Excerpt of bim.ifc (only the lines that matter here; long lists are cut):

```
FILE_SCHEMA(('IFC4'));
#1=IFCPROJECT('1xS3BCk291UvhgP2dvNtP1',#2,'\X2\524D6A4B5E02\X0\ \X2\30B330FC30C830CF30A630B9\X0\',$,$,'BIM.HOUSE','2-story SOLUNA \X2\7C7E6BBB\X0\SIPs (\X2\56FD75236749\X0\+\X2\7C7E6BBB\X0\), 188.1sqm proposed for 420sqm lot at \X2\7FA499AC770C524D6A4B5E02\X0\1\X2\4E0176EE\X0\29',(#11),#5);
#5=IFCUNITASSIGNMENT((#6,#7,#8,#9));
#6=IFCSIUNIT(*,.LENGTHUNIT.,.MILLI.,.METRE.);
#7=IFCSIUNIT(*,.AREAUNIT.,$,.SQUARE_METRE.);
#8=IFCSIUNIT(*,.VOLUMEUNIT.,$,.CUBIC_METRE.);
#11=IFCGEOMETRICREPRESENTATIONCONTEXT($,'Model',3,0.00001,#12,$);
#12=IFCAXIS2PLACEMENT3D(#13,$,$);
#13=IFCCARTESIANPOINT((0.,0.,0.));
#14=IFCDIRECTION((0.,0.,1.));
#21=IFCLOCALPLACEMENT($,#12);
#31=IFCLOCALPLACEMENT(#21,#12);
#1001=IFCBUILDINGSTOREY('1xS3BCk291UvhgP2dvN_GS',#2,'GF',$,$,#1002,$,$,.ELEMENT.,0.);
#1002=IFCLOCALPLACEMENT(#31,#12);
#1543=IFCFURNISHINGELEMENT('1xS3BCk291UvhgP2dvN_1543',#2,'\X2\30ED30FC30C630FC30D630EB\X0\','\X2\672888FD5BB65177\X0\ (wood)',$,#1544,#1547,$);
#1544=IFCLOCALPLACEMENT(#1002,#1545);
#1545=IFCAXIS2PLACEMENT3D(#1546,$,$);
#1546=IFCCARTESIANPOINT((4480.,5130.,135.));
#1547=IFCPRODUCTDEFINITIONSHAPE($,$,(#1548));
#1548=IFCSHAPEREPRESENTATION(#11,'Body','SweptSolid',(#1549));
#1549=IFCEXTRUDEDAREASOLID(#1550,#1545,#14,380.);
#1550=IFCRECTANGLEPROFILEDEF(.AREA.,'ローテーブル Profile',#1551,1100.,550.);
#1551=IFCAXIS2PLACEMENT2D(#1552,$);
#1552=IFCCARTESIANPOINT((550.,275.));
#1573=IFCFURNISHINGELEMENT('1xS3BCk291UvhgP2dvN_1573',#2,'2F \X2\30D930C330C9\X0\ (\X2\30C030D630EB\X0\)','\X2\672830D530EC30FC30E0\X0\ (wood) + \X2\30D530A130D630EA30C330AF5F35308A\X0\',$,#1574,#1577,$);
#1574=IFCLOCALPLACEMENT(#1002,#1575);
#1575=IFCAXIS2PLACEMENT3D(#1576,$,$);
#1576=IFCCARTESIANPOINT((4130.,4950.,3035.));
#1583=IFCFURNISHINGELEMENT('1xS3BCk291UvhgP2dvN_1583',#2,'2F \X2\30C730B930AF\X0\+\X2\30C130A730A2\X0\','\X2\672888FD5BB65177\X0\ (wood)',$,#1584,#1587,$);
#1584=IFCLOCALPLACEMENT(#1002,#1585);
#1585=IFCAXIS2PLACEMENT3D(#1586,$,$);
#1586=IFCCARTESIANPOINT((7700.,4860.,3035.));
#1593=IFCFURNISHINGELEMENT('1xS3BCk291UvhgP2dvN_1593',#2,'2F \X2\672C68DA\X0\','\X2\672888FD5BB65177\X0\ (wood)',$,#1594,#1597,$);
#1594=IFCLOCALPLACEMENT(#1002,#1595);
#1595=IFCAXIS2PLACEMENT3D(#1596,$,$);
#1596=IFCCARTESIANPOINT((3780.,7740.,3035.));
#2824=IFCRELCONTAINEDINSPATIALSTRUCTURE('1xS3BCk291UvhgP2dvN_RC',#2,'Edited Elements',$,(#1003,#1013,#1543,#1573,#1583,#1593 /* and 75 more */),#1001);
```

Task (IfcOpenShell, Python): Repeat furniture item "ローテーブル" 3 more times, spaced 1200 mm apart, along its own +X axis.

```python
import ifcopenshell
import ifcopenshell.api.geometry
import ifcopenshell.api.root
import ifcopenshell.util.element
import ifcopenshell.util.placement
import ifcopenshell.util.unit

model = ifcopenshell.open("bim.ifc")
unit_scale = ifcopenshell.util.unit.calculate_unit_scale(model)


def reuse_history(source, copy):
    """copy_class also copies each property set's owner history, people and application; keep the originals."""
    for rel in copy.IsDefinedBy:
        if rel.is_a("IfcRelDefinesByProperties") and (history := rel.RelatingPropertyDefinition.OwnerHistory):
            rel.RelatingPropertyDefinition.OwnerHistory = source.OwnerHistory
            ifcopenshell.util.element.remove_deep2(model, history)


source = model.by_guid("1xS3BCk291UvhgP2dvN_1543")
base = ifcopenshell.util.placement.get_local_placement(source.ObjectPlacement)
step = base[:3, 0] * 1.2 / unit_scale

for i in range(1, 4):
    copy = ifcopenshell.api.root.copy_class(model, product=source)
    copy.Representation = ifcopenshell.util.element.copy_deep(
        model, source.Representation, exclude=["IfcGeometricRepresentationContext", "IfcRepresentationMap"]
    )
    reuse_history(source, copy)
    matrix = base.copy()
    matrix[:3, 3] += i * step
    print("added at", matrix[:3, 3].round(3) + 0.0)
    ifcopenshell.api.geometry.edit_object_placement(model, product=copy, matrix=matrix, is_si=False)

model.write("bim_updated.ifc")
```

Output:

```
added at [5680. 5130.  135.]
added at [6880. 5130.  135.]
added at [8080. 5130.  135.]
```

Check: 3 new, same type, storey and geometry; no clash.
